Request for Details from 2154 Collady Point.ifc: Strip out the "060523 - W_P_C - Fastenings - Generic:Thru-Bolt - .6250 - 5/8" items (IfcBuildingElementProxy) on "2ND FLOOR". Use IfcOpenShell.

First a look at what the model holds.

```python
import ifcopenshell
import ifcopenshell.util.element

model = ifcopenshell.open("Details from 2154 Collady Point.ifc")
print(model.schema)
storey = next(s for s in model.by_type("IfcBuildingStorey") if s.Name == "2ND FLOOR")
proxies = [e for e in ifcopenshell.util.element.get_decomposition(storey) if e.is_a("IfcBuildingElementProxy")]
seen = {}
for e in proxies:
    element_type = ifcopenshell.util.element.get_type(e)
    name = element_type.Name if element_type not in (None, e) else None
    seen[name] = seen.get(name, 0) + 1
for name, count in sorted(seen.items(), key=str):
    print(count, "x", name)
```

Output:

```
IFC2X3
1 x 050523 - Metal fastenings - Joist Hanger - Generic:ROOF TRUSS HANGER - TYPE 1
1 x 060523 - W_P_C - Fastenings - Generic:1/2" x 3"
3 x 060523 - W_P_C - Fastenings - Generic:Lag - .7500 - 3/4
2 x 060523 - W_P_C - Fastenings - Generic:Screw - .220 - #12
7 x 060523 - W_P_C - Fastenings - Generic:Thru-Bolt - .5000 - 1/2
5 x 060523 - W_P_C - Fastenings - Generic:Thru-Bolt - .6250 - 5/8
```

```python
import ifcopenshell
import ifcopenshell.api.root
import ifcopenshell.util.element

model = ifcopenshell.open("Details from 2154 Collady Point.ifc")

storey = next(s for s in model.by_type("IfcBuildingStorey") if s.Name == "2ND FLOOR")
proxies = [e for e in ifcopenshell.util.element.get_decomposition(storey) if e.is_a("IfcBuildingElementProxy")]
targets = [e for e in proxies if (t := ifcopenshell.util.element.get_type(e)) not in (None, e) and t.Name == "060523 - W_P_C - Fastenings - Generic:Thru-Bolt - .6250 - 5/8"]

for e in targets:
    ifcopenshell.api.root.remove_product(model, product=e)
print(len(targets), "removed")

model.write("Details from 2154 Collady Point_rev.ifc")
```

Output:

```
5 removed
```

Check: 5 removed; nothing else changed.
